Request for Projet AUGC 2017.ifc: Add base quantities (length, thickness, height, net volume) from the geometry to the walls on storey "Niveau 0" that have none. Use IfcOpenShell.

First a look at what the model holds.

```python
import ifcopenshell
import ifcopenshell.util.element
import ifcopenshell.util.unit

model = ifcopenshell.open("Projet AUGC 2017.ifc")
print(model.schema)
for unit_type in ("LENGTHUNIT", "AREAUNIT", "VOLUMEUNIT"):
    print(unit_type, ifcopenshell.util.unit.calculate_unit_scale(model, unit_type))
storey = next(s for s in model.by_type("IfcBuildingStorey") if s.Name == "Niveau 0")
walls = [e for e in ifcopenshell.util.element.get_decomposition(storey) if e.is_a("IfcWall")]
for e in sorted(walls, key=lambda e: e.id()):
    print(e.id(), e.is_a(), e.Name, list(ifcopenshell.util.element.get_psets(e, qtos_only=True)), sep=" | ")
```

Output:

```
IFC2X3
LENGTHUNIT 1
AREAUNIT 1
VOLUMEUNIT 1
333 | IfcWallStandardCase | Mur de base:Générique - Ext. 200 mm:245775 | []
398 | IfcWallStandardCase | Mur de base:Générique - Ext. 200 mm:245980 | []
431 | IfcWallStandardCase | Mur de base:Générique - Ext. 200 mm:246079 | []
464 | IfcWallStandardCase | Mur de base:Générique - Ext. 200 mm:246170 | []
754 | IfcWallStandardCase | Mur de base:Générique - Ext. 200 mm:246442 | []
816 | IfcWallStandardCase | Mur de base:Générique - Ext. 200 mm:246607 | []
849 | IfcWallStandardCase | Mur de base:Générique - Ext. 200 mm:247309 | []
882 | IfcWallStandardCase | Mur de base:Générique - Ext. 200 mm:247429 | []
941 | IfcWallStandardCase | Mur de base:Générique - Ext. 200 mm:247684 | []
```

```python
import ifcopenshell
import ifcopenshell.api.pset
import ifcopenshell.geom
import ifcopenshell.util.element
import ifcopenshell.util.shape
import ifcopenshell.util.unit

model = ifcopenshell.open("Projet AUGC 2017.ifc")
unit_scale = ifcopenshell.util.unit.calculate_unit_scale(model)
volume_scale = ifcopenshell.util.unit.calculate_unit_scale(model, "VOLUMEUNIT")
settings = ifcopenshell.geom.settings()

storey = next(s for s in model.by_type("IfcBuildingStorey") if s.Name == "Niveau 0")
walls = [e for e in ifcopenshell.util.element.get_decomposition(storey) if e.is_a("IfcWall")]

for e in sorted(walls, key=lambda e: e.id()):
    if ifcopenshell.util.element.get_psets(e, qtos_only=True, should_inherit=False):
        continue
    # Geometry comes back in metres, in the element's own axes.
    shape = ifcopenshell.geom.create_shape(settings, e)
    values = {
        "Length": ifcopenshell.util.shape.get_x(shape.geometry) / unit_scale,
        "Width": ifcopenshell.util.shape.get_y(shape.geometry) / unit_scale,
        "Height": ifcopenshell.util.shape.get_z(shape.geometry) / unit_scale,
        "NetVolume": ifcopenshell.util.shape.get_volume(shape.geometry) / volume_scale,
    }
    qto = ifcopenshell.api.pset.add_qto(model, product=e, name="BaseQuantities")
    ifcopenshell.api.pset.edit_qto(model, qto=qto, properties=values)
    print(e.id(), {k: round(v, 3) for k, v in values.items()})

model.write("Projet AUGC 2017_rev.ifc")
```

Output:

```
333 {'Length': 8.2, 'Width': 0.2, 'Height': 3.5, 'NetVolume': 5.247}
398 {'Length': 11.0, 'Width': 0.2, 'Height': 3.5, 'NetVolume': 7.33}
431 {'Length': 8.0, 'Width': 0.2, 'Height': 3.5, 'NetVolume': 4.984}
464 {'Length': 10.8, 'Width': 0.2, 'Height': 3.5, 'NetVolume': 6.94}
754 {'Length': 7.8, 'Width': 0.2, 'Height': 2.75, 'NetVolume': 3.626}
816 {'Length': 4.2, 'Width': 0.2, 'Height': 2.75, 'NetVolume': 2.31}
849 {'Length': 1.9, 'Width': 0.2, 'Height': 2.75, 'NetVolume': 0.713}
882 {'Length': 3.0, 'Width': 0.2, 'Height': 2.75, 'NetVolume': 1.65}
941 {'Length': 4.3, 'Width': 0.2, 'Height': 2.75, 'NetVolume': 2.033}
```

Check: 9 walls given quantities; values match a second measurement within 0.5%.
